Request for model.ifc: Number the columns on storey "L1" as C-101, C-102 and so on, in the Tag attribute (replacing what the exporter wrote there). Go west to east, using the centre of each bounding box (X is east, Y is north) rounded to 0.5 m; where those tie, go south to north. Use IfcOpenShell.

First a look at what the model holds.

```python
import ifcopenshell
import ifcopenshell.util.element
import ifcopenshell.util.placement

model = ifcopenshell.open("model.ifc")
print(model.schema)
storey = next(s for s in model.by_type("IfcBuildingStorey") if s.Name == "L1")
columns = [e for e in ifcopenshell.util.element.get_decomposition(storey) if e.is_a("IfcColumn")]
for e in sorted(columns, key=lambda e: e.id()):
    origin = ifcopenshell.util.placement.get_local_placement(e.ObjectPlacement)[:3, 3]
    print(e.id(), e.Tag, e.Name, origin.round(2) + 0.0, sep=" | ")
```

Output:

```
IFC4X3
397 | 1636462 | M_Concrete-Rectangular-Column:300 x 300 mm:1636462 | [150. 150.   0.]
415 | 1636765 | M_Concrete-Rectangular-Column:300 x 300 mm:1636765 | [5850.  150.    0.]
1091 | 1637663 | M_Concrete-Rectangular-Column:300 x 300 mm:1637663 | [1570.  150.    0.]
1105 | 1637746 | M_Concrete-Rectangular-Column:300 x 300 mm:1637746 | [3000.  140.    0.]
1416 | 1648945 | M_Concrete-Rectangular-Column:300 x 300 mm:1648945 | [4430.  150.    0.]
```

```python
import ifcopenshell
import ifcopenshell.geom
import ifcopenshell.util.element
import ifcopenshell.util.shape

model = ifcopenshell.open("model.ifc")
settings = ifcopenshell.geom.settings()
settings.set("use-world-coords", True)


def centre(element):
    shape = ifcopenshell.geom.create_shape(settings, element)
    return ifcopenshell.util.shape.get_bbox_centroid(shape.geometry)


storey = next(s for s in model.by_type("IfcBuildingStorey") if s.Name == "L1")
columns = [e for e in ifcopenshell.util.element.get_decomposition(storey) if e.is_a("IfcColumn")]

# Insertion points can sit at a corner or the storey origin, so sort by the geometry (in metres).
centres = {e: centre(e) for e in columns}
columns.sort(key=lambda e: (round(centres[e][0] / 0.5), centres[e][1]))

for i, e in enumerate(columns, start=1):
    number = f"C-1{i:02d}"
    e.Tag = number
    print(e.id(), number)

model.write("model_edited.ifc")
```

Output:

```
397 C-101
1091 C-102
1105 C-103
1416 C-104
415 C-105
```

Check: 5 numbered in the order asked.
